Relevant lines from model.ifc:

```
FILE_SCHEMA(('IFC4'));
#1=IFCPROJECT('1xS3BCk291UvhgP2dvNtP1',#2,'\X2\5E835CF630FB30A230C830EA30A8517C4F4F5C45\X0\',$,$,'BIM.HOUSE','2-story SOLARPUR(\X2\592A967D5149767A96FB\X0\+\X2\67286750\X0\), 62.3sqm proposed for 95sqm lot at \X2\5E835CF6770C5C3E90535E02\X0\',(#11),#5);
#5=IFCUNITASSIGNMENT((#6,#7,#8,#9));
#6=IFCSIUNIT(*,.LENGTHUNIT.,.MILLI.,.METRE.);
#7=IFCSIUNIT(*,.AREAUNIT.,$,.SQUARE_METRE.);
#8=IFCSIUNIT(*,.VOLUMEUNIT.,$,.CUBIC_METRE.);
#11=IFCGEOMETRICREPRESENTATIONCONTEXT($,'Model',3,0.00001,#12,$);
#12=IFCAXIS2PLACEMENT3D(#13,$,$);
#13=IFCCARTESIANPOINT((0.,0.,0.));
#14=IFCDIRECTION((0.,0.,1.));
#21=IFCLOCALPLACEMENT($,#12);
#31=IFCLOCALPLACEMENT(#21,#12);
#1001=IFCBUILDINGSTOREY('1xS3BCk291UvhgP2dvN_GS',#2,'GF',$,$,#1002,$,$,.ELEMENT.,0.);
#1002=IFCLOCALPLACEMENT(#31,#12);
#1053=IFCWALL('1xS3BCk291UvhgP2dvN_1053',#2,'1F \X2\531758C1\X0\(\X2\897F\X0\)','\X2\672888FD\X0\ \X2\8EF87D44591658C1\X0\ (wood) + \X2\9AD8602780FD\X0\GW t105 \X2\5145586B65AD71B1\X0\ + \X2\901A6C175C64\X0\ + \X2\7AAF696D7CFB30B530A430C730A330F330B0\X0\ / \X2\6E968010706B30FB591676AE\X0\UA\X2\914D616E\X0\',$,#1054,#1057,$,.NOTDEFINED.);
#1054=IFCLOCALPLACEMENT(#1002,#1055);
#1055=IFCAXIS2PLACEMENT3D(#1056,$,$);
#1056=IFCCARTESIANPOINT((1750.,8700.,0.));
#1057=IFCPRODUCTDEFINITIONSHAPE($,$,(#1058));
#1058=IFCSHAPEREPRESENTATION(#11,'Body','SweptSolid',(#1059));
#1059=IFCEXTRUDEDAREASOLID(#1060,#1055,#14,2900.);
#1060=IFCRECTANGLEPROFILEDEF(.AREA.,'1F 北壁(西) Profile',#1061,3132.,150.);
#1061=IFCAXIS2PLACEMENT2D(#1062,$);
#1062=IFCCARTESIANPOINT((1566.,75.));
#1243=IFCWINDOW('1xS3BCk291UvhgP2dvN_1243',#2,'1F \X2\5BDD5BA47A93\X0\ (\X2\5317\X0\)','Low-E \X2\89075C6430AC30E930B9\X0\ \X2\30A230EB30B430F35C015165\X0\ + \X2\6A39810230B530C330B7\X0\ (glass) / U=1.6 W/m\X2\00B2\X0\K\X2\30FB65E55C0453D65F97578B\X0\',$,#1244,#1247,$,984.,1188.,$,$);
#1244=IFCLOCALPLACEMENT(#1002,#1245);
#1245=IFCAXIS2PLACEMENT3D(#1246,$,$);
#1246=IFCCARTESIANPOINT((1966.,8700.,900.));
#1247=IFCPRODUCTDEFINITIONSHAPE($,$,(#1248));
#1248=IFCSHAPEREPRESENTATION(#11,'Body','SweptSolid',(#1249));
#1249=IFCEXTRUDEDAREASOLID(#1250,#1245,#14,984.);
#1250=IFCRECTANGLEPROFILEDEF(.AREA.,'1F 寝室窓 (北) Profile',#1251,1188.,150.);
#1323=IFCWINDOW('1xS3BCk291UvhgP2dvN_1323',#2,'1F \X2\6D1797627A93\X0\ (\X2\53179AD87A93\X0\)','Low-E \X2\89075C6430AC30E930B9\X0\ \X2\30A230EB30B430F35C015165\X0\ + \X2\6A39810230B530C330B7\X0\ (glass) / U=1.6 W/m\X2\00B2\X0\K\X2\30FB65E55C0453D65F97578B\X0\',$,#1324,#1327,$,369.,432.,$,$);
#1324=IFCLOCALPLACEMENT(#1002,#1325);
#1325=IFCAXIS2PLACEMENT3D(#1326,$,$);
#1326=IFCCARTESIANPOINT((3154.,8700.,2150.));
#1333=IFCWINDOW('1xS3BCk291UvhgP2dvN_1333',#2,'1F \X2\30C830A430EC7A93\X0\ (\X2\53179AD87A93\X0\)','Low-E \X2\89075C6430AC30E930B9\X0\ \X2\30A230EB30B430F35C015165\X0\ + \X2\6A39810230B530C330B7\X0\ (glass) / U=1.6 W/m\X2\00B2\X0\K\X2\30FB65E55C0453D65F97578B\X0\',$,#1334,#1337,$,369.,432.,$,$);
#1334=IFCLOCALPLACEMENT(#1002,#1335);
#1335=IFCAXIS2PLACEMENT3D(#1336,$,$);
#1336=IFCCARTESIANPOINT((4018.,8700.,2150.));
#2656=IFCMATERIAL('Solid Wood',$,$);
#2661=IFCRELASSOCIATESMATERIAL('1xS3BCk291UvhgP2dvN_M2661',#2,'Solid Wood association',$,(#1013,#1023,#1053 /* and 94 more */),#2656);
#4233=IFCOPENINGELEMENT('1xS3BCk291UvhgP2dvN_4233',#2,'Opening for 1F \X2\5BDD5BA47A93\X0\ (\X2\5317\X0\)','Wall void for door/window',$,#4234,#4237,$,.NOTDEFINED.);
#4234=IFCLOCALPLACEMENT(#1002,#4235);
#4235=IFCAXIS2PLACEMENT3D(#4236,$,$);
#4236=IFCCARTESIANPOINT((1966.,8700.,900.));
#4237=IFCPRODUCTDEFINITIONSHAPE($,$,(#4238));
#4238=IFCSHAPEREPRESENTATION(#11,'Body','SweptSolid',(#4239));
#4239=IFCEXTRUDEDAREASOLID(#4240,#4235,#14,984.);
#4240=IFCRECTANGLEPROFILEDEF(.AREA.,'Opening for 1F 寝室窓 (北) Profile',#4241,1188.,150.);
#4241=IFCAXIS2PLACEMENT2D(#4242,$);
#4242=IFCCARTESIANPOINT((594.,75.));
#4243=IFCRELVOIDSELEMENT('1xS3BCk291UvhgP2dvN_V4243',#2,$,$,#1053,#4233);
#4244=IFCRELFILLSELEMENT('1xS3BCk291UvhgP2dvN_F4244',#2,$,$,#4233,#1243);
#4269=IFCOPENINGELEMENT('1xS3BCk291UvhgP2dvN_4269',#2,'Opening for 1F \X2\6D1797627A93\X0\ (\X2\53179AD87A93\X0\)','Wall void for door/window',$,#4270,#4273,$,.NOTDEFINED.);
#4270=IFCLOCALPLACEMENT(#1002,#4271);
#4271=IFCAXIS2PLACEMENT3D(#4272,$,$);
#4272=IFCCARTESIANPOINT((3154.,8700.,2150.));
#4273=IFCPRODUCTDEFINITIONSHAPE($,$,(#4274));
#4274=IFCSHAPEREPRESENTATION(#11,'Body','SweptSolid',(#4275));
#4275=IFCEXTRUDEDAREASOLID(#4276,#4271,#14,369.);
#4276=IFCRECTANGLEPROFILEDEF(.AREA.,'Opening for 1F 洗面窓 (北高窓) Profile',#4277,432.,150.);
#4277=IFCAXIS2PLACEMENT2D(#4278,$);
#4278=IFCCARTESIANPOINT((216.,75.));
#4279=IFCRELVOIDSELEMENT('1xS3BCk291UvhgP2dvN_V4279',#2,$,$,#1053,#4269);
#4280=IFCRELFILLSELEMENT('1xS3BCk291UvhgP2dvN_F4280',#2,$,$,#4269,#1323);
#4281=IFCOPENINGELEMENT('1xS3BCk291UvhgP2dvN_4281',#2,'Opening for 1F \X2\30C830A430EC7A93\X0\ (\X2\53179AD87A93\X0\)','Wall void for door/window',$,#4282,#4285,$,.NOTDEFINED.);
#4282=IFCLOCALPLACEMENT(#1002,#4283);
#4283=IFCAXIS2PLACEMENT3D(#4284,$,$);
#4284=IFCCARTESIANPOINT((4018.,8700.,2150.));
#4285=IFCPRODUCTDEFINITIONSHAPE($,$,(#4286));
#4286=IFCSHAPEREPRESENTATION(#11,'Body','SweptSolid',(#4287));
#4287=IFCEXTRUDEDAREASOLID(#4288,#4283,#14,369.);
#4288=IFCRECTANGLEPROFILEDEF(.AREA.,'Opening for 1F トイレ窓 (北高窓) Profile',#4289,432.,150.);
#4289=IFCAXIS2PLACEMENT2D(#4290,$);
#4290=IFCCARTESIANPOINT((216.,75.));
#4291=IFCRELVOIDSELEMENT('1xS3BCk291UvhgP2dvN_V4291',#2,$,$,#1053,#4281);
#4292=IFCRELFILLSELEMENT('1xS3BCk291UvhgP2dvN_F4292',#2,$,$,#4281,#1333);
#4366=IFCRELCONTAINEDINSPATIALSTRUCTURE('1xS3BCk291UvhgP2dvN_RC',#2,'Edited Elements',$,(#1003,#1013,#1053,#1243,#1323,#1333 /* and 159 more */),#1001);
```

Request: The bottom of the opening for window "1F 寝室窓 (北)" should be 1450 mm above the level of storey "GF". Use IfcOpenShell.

```python
import numpy as np
import ifcopenshell
import ifcopenshell.api.geometry
import ifcopenshell.geom
import ifcopenshell.util.element
import ifcopenshell.util.placement
import ifcopenshell.util.shape
import ifcopenshell.util.unit

model = ifcopenshell.open("model.ifc")
unit_scale = ifcopenshell.util.unit.calculate_unit_scale(model)

window = model.by_guid("1xS3BCk291UvhgP2dvN_1243")
opening = window.FillsVoids[0].RelatingOpeningElement
storey = ifcopenshell.util.element.get_container(window, ifc_class="IfcBuildingStorey")
level = ifcopenshell.util.placement.get_local_placement(storey.ObjectPlacement)[2, 3]

# The opening's origin need not be at the sill, so measure its lowest point.
shape = ifcopenshell.geom.create_shape(ifcopenshell.geom.settings(), opening)
bottom = ifcopenshell.util.shape.get_shape_bottom_elevation(shape, shape.geometry) / unit_scale
dz = level + 1.45 / unit_scale - bottom

shift = np.array([0.0, 0.0, dz])
# The window is not placed relative to its opening, so move both.
for product in (opening, window):
    matrix = ifcopenshell.util.placement.get_local_placement(product.ObjectPlacement)
    matrix[:3, 3] += shift
    ifcopenshell.api.geometry.edit_object_placement(model, product=product, matrix=matrix, is_si=False)

print(f"moved by {dz * unit_scale:+.3f} m")

model.write("model_v2.ifc")
```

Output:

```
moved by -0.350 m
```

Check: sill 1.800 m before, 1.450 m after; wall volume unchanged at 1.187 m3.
